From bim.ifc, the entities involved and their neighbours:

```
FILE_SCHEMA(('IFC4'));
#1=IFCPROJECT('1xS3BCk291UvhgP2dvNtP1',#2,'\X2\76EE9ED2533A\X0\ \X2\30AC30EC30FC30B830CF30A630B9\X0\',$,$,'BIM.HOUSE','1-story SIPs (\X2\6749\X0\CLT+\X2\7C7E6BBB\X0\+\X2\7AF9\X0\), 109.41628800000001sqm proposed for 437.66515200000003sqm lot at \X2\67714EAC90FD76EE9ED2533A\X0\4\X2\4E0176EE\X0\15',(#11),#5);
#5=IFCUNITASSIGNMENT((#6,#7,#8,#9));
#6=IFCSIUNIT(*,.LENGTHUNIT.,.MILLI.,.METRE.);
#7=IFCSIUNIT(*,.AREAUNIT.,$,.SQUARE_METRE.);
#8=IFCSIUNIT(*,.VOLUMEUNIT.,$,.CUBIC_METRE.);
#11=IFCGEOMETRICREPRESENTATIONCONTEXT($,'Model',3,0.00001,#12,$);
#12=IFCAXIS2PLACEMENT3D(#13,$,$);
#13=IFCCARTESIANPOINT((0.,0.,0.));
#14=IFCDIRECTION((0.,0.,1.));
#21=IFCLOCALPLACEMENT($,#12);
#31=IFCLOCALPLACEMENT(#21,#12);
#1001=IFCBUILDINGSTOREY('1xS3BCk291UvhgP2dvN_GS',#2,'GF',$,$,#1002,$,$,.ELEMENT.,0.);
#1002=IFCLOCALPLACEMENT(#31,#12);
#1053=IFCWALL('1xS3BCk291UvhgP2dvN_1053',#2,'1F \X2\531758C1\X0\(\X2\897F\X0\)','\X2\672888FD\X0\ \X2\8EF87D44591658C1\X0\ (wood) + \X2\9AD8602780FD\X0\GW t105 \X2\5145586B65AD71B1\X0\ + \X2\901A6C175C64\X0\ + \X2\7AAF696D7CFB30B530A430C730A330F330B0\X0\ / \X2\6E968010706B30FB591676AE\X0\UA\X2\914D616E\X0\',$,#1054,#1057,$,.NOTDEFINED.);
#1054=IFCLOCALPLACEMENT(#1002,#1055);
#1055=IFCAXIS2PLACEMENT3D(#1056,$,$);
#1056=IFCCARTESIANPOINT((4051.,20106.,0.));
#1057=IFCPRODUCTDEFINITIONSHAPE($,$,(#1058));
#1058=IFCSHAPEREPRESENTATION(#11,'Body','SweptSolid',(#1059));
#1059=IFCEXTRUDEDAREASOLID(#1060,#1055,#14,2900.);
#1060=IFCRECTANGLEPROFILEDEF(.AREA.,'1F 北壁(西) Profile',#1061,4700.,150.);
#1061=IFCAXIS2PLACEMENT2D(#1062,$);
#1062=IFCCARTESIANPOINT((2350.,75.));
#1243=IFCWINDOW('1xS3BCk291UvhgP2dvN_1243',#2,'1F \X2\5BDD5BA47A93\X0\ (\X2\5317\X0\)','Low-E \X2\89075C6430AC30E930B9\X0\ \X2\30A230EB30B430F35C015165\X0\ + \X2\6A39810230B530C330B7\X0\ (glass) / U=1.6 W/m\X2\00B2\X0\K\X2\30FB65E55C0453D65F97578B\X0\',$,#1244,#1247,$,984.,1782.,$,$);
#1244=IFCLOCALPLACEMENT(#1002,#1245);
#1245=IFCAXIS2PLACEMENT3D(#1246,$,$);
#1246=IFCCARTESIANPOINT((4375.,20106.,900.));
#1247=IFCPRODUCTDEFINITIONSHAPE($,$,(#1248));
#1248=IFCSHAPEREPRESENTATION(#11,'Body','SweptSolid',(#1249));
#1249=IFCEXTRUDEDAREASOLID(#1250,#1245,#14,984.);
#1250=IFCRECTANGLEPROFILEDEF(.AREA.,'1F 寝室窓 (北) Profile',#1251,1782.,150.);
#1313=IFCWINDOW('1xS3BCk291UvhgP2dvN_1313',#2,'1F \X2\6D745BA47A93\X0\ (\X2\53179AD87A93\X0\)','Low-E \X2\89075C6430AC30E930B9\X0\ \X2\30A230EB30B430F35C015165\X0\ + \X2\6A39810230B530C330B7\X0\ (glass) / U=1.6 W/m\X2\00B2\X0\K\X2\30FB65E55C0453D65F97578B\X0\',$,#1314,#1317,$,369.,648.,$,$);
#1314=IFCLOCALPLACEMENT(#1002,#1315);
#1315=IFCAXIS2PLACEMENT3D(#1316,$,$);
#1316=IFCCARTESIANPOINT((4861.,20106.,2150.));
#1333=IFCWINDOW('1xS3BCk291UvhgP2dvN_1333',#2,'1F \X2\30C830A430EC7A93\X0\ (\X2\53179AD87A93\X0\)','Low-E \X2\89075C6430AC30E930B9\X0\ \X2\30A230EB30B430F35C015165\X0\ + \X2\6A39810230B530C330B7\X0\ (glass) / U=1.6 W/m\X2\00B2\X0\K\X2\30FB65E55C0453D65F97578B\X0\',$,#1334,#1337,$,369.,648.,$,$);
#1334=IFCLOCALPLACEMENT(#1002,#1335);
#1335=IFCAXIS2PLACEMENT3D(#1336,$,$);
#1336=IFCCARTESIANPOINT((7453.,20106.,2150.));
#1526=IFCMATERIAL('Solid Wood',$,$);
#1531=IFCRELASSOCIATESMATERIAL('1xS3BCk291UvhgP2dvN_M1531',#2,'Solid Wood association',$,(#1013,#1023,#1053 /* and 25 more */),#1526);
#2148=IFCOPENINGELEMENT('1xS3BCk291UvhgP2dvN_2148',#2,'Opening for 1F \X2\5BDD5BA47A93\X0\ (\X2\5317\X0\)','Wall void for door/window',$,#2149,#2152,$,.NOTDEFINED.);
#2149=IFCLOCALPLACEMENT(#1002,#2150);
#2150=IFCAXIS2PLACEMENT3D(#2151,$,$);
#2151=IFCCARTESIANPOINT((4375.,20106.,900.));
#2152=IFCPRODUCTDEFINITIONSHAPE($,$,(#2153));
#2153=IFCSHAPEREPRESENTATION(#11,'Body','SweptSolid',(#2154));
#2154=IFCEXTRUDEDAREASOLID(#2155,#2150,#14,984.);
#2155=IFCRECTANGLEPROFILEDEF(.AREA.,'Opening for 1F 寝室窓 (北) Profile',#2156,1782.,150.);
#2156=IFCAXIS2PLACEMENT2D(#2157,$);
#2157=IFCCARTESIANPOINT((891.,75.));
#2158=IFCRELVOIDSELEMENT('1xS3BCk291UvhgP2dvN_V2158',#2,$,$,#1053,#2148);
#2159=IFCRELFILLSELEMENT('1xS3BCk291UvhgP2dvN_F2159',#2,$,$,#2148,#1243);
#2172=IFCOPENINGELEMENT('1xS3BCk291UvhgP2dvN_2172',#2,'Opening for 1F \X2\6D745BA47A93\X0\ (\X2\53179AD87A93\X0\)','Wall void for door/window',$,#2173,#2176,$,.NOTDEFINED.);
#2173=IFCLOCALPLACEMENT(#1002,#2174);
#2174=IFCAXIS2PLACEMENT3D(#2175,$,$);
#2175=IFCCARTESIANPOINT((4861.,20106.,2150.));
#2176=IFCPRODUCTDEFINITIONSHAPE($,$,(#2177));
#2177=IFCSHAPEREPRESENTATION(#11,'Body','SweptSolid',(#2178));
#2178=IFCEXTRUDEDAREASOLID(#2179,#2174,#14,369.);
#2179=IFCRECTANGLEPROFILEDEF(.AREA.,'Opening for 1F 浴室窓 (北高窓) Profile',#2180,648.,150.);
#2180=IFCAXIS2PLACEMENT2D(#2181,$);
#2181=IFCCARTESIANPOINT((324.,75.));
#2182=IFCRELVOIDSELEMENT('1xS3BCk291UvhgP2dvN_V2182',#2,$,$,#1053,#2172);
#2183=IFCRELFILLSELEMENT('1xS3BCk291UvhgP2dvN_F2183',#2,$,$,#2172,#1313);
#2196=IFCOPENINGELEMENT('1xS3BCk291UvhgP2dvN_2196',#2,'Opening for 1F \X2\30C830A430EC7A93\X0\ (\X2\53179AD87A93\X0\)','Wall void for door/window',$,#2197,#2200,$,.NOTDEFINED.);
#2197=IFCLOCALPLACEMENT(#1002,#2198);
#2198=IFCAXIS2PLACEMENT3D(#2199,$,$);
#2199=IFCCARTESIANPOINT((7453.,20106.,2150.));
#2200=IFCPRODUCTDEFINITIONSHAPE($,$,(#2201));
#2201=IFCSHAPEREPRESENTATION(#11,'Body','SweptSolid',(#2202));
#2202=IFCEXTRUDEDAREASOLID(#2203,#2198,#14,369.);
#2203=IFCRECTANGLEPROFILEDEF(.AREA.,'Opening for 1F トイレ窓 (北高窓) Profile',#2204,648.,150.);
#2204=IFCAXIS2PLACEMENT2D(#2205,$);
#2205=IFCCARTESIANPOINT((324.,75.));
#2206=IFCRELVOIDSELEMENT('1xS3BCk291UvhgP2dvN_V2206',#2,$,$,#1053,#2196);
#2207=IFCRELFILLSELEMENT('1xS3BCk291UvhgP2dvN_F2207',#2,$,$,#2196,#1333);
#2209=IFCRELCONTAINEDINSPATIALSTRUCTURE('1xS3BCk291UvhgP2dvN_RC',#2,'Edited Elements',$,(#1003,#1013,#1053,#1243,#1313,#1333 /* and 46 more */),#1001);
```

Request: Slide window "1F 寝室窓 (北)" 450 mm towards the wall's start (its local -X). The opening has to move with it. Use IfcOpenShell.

```python
import ifcopenshell
import ifcopenshell.api.geometry
import ifcopenshell.util.placement
import ifcopenshell.util.unit

model = ifcopenshell.open("bim.ifc")
unit_scale = ifcopenshell.util.unit.calculate_unit_scale(model)

window = model.by_guid("1xS3BCk291UvhgP2dvN_1243")
opening = window.FillsVoids[0].RelatingOpeningElement
wall = opening.VoidsElements[0].RelatingBuildingElement

wall_matrix = ifcopenshell.util.placement.get_local_placement(wall.ObjectPlacement)
shift = wall_matrix[:3, 0] * -0.45 / unit_scale
before = ifcopenshell.util.placement.get_local_placement(window.ObjectPlacement)[:3, 3].copy()

# The window is not placed relative to its opening, so move both.
for product in (opening, window):
    matrix = ifcopenshell.util.placement.get_local_placement(product.ObjectPlacement)
    matrix[:3, 3] += shift
    ifcopenshell.api.geometry.edit_object_placement(model, product=product, matrix=matrix, is_si=False)

after = ifcopenshell.util.placement.get_local_placement(window.ObjectPlacement)[:3, 3]
print("window moved by", (after - before).round(3) + 0.0)

model.write("bim_updated.ifc")
```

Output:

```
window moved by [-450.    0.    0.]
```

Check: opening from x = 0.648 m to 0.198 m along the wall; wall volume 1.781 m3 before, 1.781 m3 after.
